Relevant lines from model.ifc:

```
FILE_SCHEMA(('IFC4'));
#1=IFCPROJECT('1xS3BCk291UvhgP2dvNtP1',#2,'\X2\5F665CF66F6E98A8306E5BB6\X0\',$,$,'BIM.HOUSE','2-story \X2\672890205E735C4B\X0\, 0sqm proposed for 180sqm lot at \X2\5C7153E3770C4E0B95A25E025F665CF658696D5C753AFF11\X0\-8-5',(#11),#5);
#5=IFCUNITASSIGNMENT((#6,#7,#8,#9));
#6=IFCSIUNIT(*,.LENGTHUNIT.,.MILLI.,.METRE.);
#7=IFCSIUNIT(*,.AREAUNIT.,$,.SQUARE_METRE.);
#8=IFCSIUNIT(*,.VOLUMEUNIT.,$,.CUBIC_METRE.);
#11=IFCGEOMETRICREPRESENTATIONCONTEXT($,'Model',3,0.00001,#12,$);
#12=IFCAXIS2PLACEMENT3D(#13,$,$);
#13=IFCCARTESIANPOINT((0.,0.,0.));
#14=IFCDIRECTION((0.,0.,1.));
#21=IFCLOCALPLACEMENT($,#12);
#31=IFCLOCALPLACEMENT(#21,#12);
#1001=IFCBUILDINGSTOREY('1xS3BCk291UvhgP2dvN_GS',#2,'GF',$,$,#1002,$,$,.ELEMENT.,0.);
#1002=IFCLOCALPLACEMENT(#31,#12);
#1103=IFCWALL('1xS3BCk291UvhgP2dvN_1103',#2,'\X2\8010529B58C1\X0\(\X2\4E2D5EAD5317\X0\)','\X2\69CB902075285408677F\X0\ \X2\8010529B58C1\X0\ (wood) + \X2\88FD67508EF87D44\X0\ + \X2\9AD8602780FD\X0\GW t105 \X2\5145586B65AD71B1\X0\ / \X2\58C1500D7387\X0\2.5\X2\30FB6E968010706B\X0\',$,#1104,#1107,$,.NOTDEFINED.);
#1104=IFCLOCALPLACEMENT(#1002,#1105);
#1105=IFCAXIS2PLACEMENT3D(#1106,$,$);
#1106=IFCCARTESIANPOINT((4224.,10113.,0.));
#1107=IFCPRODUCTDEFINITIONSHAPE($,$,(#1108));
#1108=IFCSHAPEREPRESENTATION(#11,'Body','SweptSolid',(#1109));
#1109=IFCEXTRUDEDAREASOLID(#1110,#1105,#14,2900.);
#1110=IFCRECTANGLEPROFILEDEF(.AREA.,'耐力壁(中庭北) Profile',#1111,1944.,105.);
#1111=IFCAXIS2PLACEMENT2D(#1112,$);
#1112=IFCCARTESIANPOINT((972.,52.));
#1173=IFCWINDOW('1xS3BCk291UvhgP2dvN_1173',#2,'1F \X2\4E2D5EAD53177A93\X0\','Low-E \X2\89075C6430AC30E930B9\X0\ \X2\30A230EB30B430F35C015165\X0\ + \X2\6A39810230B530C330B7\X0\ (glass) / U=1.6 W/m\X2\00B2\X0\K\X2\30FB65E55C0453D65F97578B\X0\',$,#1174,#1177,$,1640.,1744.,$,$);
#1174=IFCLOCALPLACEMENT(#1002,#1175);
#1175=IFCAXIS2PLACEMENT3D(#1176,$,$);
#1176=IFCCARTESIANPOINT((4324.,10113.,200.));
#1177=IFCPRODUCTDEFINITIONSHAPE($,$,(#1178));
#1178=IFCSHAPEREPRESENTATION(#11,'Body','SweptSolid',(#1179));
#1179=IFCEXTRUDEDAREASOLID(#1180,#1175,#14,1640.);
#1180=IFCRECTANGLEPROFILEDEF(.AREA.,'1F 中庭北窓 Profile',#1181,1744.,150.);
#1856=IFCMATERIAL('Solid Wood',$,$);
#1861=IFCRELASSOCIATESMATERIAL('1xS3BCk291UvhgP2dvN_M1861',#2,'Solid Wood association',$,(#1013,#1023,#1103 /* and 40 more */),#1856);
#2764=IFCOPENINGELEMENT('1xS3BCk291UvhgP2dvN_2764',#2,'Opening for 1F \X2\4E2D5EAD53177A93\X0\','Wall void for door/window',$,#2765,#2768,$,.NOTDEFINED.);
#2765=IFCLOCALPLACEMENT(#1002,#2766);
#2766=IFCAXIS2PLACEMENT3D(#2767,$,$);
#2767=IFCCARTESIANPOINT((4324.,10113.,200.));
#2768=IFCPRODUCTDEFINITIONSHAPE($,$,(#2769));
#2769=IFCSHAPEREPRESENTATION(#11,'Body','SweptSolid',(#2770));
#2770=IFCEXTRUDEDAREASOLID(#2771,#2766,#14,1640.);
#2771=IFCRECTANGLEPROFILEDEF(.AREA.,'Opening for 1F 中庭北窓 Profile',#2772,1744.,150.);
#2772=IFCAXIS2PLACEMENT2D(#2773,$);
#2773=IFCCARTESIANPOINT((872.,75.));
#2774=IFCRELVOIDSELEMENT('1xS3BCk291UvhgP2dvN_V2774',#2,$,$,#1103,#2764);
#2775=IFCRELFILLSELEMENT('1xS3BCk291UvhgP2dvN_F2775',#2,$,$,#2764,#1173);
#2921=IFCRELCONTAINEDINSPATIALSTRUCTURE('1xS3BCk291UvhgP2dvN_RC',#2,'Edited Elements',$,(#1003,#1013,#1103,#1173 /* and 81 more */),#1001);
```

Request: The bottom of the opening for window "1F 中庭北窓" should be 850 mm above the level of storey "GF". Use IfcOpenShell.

```python
import numpy as np
import ifcopenshell
import ifcopenshell.api.geometry
import ifcopenshell.geom
import ifcopenshell.util.element
import ifcopenshell.util.placement
import ifcopenshell.util.shape
import ifcopenshell.util.unit

model = ifcopenshell.open("model.ifc")
unit_scale = ifcopenshell.util.unit.calculate_unit_scale(model)

window = model.by_id(1173)
opening = window.FillsVoids[0].RelatingOpeningElement
storey = ifcopenshell.util.element.get_container(window, ifc_class="IfcBuildingStorey")
level = ifcopenshell.util.placement.get_local_placement(storey.ObjectPlacement)[2, 3]

# The opening's origin need not be at the sill, so measure its lowest point.
shape = ifcopenshell.geom.create_shape(ifcopenshell.geom.settings(), opening)
bottom = ifcopenshell.util.shape.get_shape_bottom_elevation(shape, shape.geometry) / unit_scale
dz = level + 850.0 - bottom

shift = np.array([0.0, 0.0, dz])
# The window is not placed relative to its opening, so move both.
for product in (opening, window):
    matrix = ifcopenshell.util.placement.get_local_placement(product.ObjectPlacement)
    matrix[:3, 3] += shift
    ifcopenshell.api.geometry.edit_object_placement(model, product=product, matrix=matrix, is_si=False)

print(f"moved by {dz * unit_scale:+.3f} m")

model.write("model_updated.ifc")
```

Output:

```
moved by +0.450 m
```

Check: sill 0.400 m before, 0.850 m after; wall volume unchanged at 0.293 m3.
